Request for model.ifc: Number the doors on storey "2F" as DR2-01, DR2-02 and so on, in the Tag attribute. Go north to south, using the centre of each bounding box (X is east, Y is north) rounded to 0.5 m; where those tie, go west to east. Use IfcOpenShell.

First a look at what the model holds.

```python
import ifcopenshell
import ifcopenshell.util.element
import ifcopenshell.util.placement

model = ifcopenshell.open("model.ifc")
print(model.schema)
storey = next(s for s in model.by_type("IfcBuildingStorey") if s.Name == "2F")
doors = [e for e in ifcopenshell.util.element.get_decomposition(storey) if e.is_a("IfcDoor")]
for e in sorted(doors, key=lambda e: e.id()):
    origin = ifcopenshell.util.placement.get_local_placement(e.ObjectPlacement)[:3, 3]
    print(e.id(), e.Tag, e.Name, origin.round(2) + 0.0, sep=" | ")
```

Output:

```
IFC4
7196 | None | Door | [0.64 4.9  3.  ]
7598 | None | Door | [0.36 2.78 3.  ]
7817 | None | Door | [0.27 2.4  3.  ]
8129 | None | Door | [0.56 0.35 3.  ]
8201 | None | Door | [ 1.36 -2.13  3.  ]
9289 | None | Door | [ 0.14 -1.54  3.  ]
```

```python
import ifcopenshell
import ifcopenshell.geom
import ifcopenshell.util.element
import ifcopenshell.util.shape

model = ifcopenshell.open("model.ifc")
settings = ifcopenshell.geom.settings()
settings.set("use-world-coords", True)


def centre(element):
    shape = ifcopenshell.geom.create_shape(settings, element)
    return ifcopenshell.util.shape.get_bbox_centroid(shape.geometry)


storey = next(s for s in model.by_type("IfcBuildingStorey") if s.Name == "2F")
doors = [e for e in ifcopenshell.util.element.get_decomposition(storey) if e.is_a("IfcDoor")]

# Insertion points can sit at a corner or the storey origin, so sort by the geometry (in metres).
centres = {e: centre(e) for e in doors}
doors.sort(key=lambda e: (-round(centres[e][1] / 0.5), centres[e][0]))

for i, e in enumerate(doors, start=1):
    number = f"DR2-{i:02d}"
    e.Tag = number
    print(e.id(), number)

model.write("model_edited.ifc")
```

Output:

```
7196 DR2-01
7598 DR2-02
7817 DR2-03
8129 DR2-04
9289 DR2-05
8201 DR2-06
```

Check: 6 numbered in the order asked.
